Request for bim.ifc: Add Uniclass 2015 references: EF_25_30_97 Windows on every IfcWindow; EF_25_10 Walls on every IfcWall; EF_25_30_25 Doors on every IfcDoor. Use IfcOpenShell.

First a look at what the model holds.

```python
import ifcopenshell

model = ifcopenshell.open("bim.ifc")
print(model.schema)
print("classifications:", [c.Name for c in model.by_type("IfcClassification")])
for ifc_class in ("IfcDoor", "IfcRoof", "IfcStair", "IfcWall", "IfcWindow"):
    print(ifc_class, len(model.by_type(ifc_class)))
```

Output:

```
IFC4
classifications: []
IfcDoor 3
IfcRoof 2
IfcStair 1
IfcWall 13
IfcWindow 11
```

```python
import ifcopenshell
import ifcopenshell.api.classification

model = ifcopenshell.open("bim.ifc")

system = ifcopenshell.api.classification.add_classification(model, classification="Uniclass 2015")

codes = {
    "IfcWindow": ("EF_25_30_97", "Windows"),
    "IfcWall": ("EF_25_10", "Walls"),
    "IfcDoor": ("EF_25_30_25", "Doors"),
}
for ifc_class, (code, name) in codes.items():
    products = model.by_type(ifc_class)
    ifcopenshell.api.classification.add_reference(
        model, products=products, classification=system, identification=code, name=name
    )
    print(code, len(products))

model.write("bim-out.ifc")
```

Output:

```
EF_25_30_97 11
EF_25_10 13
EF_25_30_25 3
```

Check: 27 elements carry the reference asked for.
